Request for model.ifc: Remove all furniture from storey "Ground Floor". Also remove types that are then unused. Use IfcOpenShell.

First a look at what the model holds.

```python
import ifcopenshell
import ifcopenshell.util.element

model = ifcopenshell.open("model.ifc")
print(model.schema)
storey = next(s for s in model.by_type("IfcBuildingStorey") if s.Name == "Ground Floor")
furniture = [e for e in ifcopenshell.util.element.get_decomposition(storey) if e.is_a("IfcFurnishingElement")]
seen = {}
for e in furniture:
    element_type = ifcopenshell.util.element.get_type(e)
    name = element_type.Name if element_type not in (None, e) else None
    seen[name] = seen.get(name, 0) + 1
for name, count in sorted(seen.items(), key=str):
    print(count, "x", name)
```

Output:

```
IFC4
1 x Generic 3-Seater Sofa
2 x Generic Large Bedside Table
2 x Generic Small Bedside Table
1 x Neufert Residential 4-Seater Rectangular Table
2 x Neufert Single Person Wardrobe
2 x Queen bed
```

```python
import ifcopenshell
import ifcopenshell.api.root
import ifcopenshell.util.element

model = ifcopenshell.open("model.ifc")

storey = next(s for s in model.by_type("IfcBuildingStorey") if s.Name == "Ground Floor")
furniture = [e for e in ifcopenshell.util.element.get_decomposition(storey) if e.is_a("IfcFurnishingElement")]
types = {ifcopenshell.util.element.get_type(e) for e in furniture} - {None, *furniture}

for e in furniture:
    ifcopenshell.api.root.remove_product(model, product=e)
print(len(furniture), "removed")

unused = [t for t in types if not ifcopenshell.util.element.get_types(t)]
for t in unused:
    ifcopenshell.api.root.remove_product(model, product=t)
print(len(unused), "unused types removed")

model.write("model_edited.ifc")
```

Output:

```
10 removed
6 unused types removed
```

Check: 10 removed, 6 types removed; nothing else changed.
